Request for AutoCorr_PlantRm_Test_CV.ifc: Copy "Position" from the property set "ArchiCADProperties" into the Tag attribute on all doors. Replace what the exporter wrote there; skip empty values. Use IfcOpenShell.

First a look at what the model holds.

```python
import ifcopenshell
import ifcopenshell.util.element

model = ifcopenshell.open("AutoCorr_PlantRm_Test_CV.ifc")
print(model.schema)
doors = model.by_type("IfcDoor")
print(len(doors), "doors")
for e in doors[:8]:
    source = ifcopenshell.util.element.get_pset(e, "ArchiCADProperties", "Position")
    target = e.Tag
    print(e.id(), repr(source), repr(target), sep=" | ")
```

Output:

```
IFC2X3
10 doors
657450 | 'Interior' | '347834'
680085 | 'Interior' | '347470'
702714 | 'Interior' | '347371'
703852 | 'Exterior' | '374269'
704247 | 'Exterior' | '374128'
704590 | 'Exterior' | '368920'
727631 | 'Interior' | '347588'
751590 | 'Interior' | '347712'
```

```python
import ifcopenshell
import ifcopenshell.util.element

model = ifcopenshell.open("AutoCorr_PlantRm_Test_CV.ifc")

count = 0
for e in model.by_type("IfcDoor"):
    value = ifcopenshell.util.element.get_pset(e, "ArchiCADProperties", "Position")
    current = e.Tag
    if not value or not value.strip() or current == value:
        continue
    e.Tag = value
    count += 1

print(count, "doors updated")

model.write("AutoCorr_PlantRm_Test_CV_v2.ifc")
```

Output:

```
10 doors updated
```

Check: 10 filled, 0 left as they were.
